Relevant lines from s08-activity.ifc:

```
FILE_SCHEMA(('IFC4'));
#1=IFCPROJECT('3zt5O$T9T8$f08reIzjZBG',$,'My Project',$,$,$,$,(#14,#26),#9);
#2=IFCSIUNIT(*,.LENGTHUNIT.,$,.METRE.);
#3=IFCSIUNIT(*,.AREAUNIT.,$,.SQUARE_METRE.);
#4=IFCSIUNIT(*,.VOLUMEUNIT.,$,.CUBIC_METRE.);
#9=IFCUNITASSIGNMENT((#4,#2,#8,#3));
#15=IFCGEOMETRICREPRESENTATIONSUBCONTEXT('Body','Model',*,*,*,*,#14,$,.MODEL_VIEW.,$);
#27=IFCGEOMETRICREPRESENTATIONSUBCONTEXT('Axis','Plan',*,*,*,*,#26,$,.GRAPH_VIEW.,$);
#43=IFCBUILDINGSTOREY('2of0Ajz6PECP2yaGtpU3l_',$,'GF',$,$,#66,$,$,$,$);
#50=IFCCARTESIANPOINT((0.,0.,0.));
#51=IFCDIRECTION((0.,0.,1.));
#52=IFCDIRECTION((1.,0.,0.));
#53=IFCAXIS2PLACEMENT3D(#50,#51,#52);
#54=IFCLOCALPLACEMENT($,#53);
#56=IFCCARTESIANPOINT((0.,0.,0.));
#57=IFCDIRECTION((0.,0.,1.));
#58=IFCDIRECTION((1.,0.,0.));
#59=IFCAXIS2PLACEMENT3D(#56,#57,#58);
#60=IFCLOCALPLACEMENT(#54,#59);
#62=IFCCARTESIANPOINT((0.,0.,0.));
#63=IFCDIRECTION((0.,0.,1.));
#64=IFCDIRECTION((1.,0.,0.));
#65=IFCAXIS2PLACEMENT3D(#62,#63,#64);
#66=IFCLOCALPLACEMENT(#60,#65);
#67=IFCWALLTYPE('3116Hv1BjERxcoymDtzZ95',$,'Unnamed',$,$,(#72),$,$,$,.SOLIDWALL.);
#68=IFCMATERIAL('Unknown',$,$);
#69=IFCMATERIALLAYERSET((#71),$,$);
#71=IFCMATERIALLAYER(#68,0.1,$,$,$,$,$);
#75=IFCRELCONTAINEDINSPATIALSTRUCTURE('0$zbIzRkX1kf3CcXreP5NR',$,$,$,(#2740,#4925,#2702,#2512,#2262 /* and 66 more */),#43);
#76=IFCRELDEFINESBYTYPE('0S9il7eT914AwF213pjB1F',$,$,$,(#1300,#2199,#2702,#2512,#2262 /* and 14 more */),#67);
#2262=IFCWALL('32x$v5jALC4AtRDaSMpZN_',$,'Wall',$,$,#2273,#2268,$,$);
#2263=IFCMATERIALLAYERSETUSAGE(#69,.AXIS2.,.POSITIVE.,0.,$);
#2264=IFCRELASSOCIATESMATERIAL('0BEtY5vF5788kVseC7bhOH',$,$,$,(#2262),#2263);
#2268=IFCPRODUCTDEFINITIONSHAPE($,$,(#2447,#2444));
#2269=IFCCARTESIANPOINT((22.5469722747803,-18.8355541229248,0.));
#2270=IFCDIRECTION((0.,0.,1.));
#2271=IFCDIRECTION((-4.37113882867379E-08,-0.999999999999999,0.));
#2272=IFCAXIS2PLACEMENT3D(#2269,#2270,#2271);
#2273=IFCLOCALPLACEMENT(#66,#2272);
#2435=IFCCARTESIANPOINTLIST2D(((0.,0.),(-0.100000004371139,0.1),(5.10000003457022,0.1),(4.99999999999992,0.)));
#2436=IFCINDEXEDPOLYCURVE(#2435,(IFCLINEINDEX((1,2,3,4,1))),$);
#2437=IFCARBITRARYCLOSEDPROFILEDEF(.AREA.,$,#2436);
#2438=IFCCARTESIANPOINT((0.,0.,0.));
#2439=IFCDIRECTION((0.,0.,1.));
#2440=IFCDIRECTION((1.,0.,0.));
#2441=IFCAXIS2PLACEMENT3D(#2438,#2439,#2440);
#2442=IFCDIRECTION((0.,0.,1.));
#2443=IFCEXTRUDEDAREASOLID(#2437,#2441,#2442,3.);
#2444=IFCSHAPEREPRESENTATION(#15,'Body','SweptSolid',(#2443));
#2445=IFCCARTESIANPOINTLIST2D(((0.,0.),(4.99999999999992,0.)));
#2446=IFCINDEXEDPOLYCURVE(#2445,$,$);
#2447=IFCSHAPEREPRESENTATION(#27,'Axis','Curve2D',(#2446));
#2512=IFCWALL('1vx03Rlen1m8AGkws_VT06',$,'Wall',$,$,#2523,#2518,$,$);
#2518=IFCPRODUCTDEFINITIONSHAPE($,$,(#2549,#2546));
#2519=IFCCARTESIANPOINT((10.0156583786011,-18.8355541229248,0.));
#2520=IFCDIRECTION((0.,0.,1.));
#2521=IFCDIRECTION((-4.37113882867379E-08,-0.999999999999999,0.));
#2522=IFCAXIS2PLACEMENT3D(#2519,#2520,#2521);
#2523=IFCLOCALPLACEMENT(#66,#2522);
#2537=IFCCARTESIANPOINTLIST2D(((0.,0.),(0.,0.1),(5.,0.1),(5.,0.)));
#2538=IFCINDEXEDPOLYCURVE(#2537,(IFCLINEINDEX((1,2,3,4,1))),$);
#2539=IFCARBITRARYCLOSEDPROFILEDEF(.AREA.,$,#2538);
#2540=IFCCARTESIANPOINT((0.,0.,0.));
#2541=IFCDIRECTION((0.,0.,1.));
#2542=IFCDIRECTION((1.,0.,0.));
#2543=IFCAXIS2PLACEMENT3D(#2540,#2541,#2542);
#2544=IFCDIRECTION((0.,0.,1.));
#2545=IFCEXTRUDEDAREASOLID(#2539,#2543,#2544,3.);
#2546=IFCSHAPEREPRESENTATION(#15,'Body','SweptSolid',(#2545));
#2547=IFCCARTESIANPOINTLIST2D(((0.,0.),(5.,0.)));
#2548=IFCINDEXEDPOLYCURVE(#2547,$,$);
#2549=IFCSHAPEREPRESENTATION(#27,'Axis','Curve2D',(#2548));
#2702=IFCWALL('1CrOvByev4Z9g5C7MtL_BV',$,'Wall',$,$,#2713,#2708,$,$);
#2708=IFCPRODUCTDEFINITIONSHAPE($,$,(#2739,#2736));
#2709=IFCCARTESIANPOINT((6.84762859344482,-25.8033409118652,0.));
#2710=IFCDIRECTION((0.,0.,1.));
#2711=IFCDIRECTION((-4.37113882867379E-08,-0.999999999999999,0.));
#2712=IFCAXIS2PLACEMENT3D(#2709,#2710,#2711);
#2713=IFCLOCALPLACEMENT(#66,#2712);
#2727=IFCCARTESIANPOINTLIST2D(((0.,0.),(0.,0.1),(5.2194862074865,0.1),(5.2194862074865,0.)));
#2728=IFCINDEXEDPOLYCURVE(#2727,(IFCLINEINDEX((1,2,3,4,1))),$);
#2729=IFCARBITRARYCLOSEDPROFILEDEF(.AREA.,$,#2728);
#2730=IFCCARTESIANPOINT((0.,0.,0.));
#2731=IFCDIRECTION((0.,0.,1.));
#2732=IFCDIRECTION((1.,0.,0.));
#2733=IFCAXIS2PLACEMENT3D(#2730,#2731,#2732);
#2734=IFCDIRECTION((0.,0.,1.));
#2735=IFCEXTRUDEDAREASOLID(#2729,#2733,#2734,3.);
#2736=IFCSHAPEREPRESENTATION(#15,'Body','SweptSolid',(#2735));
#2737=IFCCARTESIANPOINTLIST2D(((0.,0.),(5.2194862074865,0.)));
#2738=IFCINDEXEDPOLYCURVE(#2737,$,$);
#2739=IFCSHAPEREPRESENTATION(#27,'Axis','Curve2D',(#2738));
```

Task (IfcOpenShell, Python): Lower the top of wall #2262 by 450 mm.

```python
import ifcopenshell
import ifcopenshell.geom
import ifcopenshell.util.representation
import ifcopenshell.util.shape
import ifcopenshell.util.unit

model = ifcopenshell.open("s08-activity.ifc")
unit_scale = ifcopenshell.util.unit.calculate_unit_scale(model)
settings = ifcopenshell.geom.settings()


def volume(element):
    """Net volume in cubic metres, openings subtracted."""
    shape = ifcopenshell.geom.create_shape(settings, element)
    return ifcopenshell.util.shape.get_volume(shape.geometry)


wall = model.by_guid("32x$v5jALC4AtRDaSMpZN_")
before = volume(wall)

body = ifcopenshell.util.representation.get_representation(wall, "Model", "Body")
solid = body.Items[0]
old_height = solid.Depth
solid.Depth -= 0.45 / unit_scale
after = volume(wall)

print(f"height {old_height:g} -> {solid.Depth:g}, volume {before:.3f} -> {after:.3f} m3")

model.write("s08-activity_v2.ifc")
```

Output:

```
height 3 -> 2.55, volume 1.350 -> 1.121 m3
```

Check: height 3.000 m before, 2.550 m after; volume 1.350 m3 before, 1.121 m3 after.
